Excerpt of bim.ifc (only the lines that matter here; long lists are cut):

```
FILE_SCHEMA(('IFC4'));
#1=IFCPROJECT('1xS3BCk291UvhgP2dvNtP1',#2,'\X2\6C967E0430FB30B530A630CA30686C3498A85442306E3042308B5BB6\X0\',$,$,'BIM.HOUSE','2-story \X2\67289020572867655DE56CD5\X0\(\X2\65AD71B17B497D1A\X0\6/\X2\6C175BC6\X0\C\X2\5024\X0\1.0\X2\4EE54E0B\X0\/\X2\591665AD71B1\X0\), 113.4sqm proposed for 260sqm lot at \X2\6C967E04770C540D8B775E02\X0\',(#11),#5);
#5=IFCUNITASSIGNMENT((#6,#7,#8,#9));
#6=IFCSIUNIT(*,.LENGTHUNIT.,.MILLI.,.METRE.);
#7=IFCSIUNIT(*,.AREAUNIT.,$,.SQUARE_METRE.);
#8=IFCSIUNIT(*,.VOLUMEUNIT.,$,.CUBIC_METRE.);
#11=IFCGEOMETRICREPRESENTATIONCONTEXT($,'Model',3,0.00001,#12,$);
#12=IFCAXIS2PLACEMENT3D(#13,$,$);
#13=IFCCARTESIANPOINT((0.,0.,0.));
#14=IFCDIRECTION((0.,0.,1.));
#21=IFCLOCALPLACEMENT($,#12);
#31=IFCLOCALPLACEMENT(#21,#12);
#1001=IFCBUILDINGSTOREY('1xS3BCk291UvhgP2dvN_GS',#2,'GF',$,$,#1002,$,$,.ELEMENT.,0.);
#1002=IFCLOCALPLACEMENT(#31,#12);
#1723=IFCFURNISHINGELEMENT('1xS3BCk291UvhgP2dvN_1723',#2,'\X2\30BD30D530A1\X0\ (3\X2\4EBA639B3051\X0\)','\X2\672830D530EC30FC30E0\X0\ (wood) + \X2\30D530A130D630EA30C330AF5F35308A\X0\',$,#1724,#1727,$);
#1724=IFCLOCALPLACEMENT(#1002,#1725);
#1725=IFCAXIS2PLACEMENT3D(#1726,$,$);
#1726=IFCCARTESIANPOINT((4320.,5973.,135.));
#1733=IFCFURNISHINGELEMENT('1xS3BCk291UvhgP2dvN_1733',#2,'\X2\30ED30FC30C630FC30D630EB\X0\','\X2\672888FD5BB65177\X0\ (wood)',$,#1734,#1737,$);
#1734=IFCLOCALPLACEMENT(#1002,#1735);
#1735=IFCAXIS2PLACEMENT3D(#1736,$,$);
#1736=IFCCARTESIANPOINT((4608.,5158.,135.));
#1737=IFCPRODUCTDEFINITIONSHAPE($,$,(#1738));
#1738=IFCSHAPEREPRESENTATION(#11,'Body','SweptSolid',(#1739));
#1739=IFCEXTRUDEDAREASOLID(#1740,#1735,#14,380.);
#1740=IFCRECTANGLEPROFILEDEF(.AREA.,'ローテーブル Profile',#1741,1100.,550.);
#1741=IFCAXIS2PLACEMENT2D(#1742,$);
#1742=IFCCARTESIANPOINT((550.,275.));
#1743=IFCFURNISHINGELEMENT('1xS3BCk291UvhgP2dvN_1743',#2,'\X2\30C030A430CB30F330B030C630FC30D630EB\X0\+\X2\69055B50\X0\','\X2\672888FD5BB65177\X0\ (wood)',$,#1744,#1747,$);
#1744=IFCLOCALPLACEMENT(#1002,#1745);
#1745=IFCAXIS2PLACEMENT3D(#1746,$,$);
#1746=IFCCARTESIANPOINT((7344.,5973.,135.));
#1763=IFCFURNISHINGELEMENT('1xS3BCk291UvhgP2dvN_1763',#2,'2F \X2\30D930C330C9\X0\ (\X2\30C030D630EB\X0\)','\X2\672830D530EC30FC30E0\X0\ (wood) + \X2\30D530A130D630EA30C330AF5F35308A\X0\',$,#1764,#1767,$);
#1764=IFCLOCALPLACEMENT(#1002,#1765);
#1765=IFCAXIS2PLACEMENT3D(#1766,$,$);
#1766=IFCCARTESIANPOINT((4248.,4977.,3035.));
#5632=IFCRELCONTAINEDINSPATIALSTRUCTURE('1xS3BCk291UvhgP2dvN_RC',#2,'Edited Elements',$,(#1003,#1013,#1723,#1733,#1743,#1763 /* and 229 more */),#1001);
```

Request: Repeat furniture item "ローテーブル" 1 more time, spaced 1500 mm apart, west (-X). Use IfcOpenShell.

```python
import numpy as np
import ifcopenshell
import ifcopenshell.api.geometry
import ifcopenshell.api.root
import ifcopenshell.util.element
import ifcopenshell.util.placement
import ifcopenshell.util.unit

model = ifcopenshell.open("bim.ifc")
unit_scale = ifcopenshell.util.unit.calculate_unit_scale(model)


def reuse_history(source, copy):
    """copy_class also copies each property set's owner history, people and application; keep the originals."""
    for rel in copy.IsDefinedBy:
        if rel.is_a("IfcRelDefinesByProperties") and (history := rel.RelatingPropertyDefinition.OwnerHistory):
            rel.RelatingPropertyDefinition.OwnerHistory = source.OwnerHistory
            ifcopenshell.util.element.remove_deep2(model, history)


source = model.by_guid("1xS3BCk291UvhgP2dvN_1733")
base = ifcopenshell.util.placement.get_local_placement(source.ObjectPlacement)
step = np.array([-1.0, 0.0, 0.0]) * 1.5 / unit_scale

for i in range(1, 2):
    copy = ifcopenshell.api.root.copy_class(model, product=source)
    copy.Representation = ifcopenshell.util.element.copy_deep(
        model, source.Representation, exclude=["IfcGeometricRepresentationContext", "IfcRepresentationMap"]
    )
    reuse_history(source, copy)
    matrix = base.copy()
    matrix[:3, 3] += i * step
    print("added at", matrix[:3, 3].round(3) + 0.0)
    ifcopenshell.api.geometry.edit_object_placement(model, product=copy, matrix=matrix, is_si=False)

model.write("bim_v2.ifc")
```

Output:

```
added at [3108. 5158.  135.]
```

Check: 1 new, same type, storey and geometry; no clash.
